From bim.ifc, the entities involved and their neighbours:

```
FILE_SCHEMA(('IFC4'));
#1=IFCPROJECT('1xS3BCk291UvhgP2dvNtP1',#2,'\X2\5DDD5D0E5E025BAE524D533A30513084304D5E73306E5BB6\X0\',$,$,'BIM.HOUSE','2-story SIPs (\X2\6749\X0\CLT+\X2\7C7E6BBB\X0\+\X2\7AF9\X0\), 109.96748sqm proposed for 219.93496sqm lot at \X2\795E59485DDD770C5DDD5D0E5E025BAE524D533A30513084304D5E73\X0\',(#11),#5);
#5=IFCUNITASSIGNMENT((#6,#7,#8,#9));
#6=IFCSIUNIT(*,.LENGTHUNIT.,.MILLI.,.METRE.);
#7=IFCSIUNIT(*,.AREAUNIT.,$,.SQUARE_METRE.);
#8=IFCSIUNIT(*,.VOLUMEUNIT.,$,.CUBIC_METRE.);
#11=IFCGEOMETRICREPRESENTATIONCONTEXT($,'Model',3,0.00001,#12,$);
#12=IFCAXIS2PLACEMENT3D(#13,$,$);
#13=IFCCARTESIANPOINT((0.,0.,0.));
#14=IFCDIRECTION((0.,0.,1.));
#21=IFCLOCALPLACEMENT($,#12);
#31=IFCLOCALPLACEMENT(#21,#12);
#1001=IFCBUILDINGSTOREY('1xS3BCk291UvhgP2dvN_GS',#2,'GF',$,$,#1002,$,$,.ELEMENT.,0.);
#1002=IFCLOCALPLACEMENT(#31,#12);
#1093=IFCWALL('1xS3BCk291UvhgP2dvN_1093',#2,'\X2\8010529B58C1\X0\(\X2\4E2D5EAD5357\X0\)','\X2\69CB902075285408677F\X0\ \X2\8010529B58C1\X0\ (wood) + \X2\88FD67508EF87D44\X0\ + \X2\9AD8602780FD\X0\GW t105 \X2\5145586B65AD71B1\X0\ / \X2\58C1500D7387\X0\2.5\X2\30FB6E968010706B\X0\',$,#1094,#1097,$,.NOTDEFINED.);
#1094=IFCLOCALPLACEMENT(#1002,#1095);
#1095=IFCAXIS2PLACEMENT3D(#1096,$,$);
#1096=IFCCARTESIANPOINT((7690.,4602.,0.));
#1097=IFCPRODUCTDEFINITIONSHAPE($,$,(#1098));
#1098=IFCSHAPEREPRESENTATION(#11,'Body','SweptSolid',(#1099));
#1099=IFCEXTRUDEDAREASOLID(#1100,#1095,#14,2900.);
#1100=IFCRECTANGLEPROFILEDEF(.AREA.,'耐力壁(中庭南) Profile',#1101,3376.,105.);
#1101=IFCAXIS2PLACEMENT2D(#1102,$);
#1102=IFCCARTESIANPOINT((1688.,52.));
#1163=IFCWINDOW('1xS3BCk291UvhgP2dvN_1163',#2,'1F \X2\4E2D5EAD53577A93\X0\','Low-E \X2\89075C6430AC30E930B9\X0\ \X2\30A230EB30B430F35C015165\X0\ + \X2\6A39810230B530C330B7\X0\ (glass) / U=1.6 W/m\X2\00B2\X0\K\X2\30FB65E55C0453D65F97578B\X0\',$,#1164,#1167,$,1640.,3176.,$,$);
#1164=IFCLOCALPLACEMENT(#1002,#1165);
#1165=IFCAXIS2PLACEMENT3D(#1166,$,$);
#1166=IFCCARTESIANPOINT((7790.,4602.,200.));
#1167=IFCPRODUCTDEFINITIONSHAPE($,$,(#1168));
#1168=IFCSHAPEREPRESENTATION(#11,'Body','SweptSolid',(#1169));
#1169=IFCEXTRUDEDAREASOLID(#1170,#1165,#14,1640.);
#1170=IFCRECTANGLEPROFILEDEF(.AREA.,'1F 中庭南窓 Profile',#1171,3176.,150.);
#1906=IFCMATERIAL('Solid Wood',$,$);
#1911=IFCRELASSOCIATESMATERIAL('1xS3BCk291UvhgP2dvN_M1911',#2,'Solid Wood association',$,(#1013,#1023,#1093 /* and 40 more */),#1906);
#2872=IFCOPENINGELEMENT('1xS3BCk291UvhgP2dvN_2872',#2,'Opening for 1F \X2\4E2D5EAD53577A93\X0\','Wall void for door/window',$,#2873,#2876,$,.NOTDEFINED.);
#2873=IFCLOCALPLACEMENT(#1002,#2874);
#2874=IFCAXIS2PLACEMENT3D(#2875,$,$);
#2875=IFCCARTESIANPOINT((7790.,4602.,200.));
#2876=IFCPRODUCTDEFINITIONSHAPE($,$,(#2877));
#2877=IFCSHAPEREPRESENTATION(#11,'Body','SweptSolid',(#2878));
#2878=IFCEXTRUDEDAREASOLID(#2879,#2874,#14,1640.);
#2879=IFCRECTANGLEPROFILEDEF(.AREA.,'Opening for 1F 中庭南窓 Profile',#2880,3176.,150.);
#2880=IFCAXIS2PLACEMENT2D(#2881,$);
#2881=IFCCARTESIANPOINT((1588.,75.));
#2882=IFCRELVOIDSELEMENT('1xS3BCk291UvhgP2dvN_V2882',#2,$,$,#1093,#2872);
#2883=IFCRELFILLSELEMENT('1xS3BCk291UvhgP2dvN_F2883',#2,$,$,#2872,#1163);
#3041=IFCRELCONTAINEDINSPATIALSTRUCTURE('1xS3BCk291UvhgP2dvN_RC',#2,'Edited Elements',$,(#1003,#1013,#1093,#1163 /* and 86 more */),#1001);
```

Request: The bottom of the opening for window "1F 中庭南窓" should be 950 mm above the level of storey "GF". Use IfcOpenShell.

```python
import numpy as np
import ifcopenshell
import ifcopenshell.api.geometry
import ifcopenshell.geom
import ifcopenshell.util.element
import ifcopenshell.util.placement
import ifcopenshell.util.shape
import ifcopenshell.util.unit

model = ifcopenshell.open("bim.ifc")
unit_scale = ifcopenshell.util.unit.calculate_unit_scale(model)

window = model.by_guid("1xS3BCk291UvhgP2dvN_1163")
opening = window.FillsVoids[0].RelatingOpeningElement
storey = ifcopenshell.util.element.get_container(window, ifc_class="IfcBuildingStorey")
level = ifcopenshell.util.placement.get_local_placement(storey.ObjectPlacement)[2, 3]

# The opening's origin need not be at the sill, so measure its lowest point.
shape = ifcopenshell.geom.create_shape(ifcopenshell.geom.settings(), opening)
bottom = ifcopenshell.util.shape.get_shape_bottom_elevation(shape, shape.geometry) / unit_scale
dz = level + 0.95 / unit_scale - bottom

shift = np.array([0.0, 0.0, dz])
# The window is not placed relative to its opening, so move both.
for product in (opening, window):
    matrix = ifcopenshell.util.placement.get_local_placement(product.ObjectPlacement)
    matrix[:3, 3] += shift
    ifcopenshell.api.geometry.edit_object_placement(model, product=product, matrix=matrix, is_si=False)

print(f"moved by {dz * unit_scale:+.3f} m")

model.write("bim_edited.ifc")
```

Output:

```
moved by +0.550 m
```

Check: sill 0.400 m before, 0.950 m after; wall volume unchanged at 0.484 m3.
